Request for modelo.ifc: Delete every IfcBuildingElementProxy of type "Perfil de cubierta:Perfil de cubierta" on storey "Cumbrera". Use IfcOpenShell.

First a look at what the model holds.

```python
import ifcopenshell
import ifcopenshell.util.element

model = ifcopenshell.open("modelo.ifc")
print(model.schema)
storey = next(s for s in model.by_type("IfcBuildingStorey") if s.Name == "Cumbrera")
proxies = [e for e in ifcopenshell.util.element.get_decomposition(storey) if e.is_a("IfcBuildingElementProxy")]
seen = {}
for e in proxies:
    element_type = ifcopenshell.util.element.get_type(e)
    name = element_type.Name if element_type not in (None, e) else None
    seen[name] = seen.get(name, 0) + 1
for name, count in sorted(seen.items(), key=str):
    print(count, "x", name)
```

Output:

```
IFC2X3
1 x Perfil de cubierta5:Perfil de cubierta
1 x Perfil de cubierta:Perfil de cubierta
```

```python
import ifcopenshell
import ifcopenshell.api.root
import ifcopenshell.util.element

model = ifcopenshell.open("modelo.ifc")

storey = next(s for s in model.by_type("IfcBuildingStorey") if s.Name == "Cumbrera")
proxies = [e for e in ifcopenshell.util.element.get_decomposition(storey) if e.is_a("IfcBuildingElementProxy")]
targets = [e for e in proxies if (t := ifcopenshell.util.element.get_type(e)) not in (None, e) and t.Name == "Perfil de cubierta:Perfil de cubierta"]

for e in targets:
    ifcopenshell.api.root.remove_product(model, product=e)
print(len(targets), "removed")

model.write("modelo_edited.ifc")
```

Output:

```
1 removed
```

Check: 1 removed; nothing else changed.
